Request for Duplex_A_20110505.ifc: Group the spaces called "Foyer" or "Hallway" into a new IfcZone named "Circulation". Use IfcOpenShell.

First a look at what the model holds.

```python
import ifcopenshell

model = ifcopenshell.open("Duplex_A_20110505.ifc")
print(model.schema)
seen = {}
for space in model.by_type("IfcSpace"):
    seen[space.LongName] = seen.get(space.LongName, 0) + 1
for name, count in sorted(seen.items(), key=str):
    print(count, "x", name)
print("zones:", [z.Name for z in model.by_type("IfcZone")][:20])
```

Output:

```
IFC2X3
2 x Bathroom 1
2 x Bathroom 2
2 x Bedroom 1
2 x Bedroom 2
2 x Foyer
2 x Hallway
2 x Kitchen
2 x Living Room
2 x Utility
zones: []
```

```python
import ifcopenshell
import ifcopenshell.api.group
import ifcopenshell.api.root

model = ifcopenshell.open("Duplex_A_20110505.ifc")

names = {"Foyer", "Hallway"}
spaces = [s for s in model.by_type("IfcSpace") if s.LongName in names]

zone = ifcopenshell.api.root.create_entity(model, ifc_class="IfcZone", name="Circulation")
ifcopenshell.api.group.assign_group(model, products=spaces, group=zone)
print(len(spaces), "spaces in", zone.Name)

model.write("Duplex_A_20110505_updated.ifc")
```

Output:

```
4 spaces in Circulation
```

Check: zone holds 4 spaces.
